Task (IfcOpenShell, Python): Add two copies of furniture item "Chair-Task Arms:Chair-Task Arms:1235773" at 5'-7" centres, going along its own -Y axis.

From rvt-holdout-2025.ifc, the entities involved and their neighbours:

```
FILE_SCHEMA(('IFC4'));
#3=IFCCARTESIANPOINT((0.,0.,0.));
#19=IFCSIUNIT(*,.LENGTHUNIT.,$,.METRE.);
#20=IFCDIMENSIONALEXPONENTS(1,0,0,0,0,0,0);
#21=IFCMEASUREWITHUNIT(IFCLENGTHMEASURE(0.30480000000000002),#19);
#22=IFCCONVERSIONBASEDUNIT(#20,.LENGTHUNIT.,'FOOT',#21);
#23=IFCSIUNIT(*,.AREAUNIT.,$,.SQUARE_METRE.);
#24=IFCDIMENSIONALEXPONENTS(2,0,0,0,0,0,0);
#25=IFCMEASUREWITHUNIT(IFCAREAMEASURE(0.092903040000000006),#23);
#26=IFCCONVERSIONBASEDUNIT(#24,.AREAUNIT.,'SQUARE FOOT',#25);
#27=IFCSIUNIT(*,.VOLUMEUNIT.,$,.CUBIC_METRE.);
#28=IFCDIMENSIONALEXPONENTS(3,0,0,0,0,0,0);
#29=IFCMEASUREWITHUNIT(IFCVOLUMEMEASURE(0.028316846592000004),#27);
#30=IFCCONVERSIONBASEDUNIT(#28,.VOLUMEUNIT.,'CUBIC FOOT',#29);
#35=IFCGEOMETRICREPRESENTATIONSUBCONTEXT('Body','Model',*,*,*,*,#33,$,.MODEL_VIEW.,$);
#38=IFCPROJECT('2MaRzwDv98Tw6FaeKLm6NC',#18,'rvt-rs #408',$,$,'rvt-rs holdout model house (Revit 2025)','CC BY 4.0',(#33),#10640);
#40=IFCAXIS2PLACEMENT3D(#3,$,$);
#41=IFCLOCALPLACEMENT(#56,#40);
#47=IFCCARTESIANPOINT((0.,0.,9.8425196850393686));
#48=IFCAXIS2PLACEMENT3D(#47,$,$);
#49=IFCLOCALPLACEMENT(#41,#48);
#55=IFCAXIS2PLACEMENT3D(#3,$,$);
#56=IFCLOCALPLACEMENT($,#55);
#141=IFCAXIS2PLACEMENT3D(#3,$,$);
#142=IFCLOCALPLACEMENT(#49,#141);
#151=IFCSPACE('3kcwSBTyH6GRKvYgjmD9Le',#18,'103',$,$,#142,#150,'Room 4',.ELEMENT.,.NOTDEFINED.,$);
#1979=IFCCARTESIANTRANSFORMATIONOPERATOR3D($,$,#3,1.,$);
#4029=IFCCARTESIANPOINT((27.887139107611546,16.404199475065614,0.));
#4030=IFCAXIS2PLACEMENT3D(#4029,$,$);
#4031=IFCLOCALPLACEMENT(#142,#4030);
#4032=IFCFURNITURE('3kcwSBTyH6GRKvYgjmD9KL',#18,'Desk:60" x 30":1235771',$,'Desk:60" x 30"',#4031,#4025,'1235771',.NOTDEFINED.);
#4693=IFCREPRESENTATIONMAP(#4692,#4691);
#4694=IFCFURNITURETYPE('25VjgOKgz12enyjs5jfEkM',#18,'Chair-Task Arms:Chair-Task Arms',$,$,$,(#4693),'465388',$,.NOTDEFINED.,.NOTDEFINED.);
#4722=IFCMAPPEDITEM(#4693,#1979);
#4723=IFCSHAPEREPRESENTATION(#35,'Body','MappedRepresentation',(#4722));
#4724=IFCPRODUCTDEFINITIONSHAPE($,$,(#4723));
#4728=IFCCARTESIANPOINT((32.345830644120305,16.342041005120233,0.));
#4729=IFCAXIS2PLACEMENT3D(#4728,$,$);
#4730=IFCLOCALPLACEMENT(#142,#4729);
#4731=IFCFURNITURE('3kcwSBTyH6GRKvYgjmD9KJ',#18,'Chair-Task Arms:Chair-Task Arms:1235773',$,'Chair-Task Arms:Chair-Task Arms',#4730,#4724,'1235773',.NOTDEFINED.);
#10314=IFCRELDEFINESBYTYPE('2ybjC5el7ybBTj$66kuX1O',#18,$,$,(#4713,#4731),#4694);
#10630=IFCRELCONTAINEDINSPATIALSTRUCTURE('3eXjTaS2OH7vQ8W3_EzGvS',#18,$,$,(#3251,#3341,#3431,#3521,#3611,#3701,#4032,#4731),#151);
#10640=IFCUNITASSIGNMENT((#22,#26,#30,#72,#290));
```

```python
import ifcopenshell
import ifcopenshell.api.geometry
import ifcopenshell.api.root
import ifcopenshell.util.element
import ifcopenshell.util.placement
import ifcopenshell.util.unit

model = ifcopenshell.open("rvt-holdout-2025.ifc")
unit_scale = ifcopenshell.util.unit.calculate_unit_scale(model)


def reuse_history(source, copy):
    """copy_class also copies each property set's owner history, people and application; keep the originals."""
    for rel in copy.IsDefinedBy:
        if rel.is_a("IfcRelDefinesByProperties") and (history := rel.RelatingPropertyDefinition.OwnerHistory):
            rel.RelatingPropertyDefinition.OwnerHistory = source.OwnerHistory
            ifcopenshell.util.element.remove_deep2(model, history)


source = model.by_guid("3kcwSBTyH6GRKvYgjmD9KJ")
base = ifcopenshell.util.placement.get_local_placement(source.ObjectPlacement)
step = -base[:3, 1] * 67 * 0.0254 / unit_scale

for i in range(1, 3):
    copy = ifcopenshell.api.root.copy_class(model, product=source)
    copy.Representation = ifcopenshell.util.element.copy_deep(
        model, source.Representation, exclude=["IfcGeometricRepresentationContext", "IfcRepresentationMap"]
    )
    copy.Name = "Chair-Task Arms:Chair-Task Arms"
    copy.Tag = None
    reuse_history(source, copy)
    matrix = base.copy()
    matrix[:3, 3] += i * step
    print("added at", matrix[:3, 3].round(3) + 0.0)
    ifcopenshell.api.geometry.edit_object_placement(model, product=copy, matrix=matrix, is_si=False)

model.write("rvt-holdout-2025_rev.ifc")
```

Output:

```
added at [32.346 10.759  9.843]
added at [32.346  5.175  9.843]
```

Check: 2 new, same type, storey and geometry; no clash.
